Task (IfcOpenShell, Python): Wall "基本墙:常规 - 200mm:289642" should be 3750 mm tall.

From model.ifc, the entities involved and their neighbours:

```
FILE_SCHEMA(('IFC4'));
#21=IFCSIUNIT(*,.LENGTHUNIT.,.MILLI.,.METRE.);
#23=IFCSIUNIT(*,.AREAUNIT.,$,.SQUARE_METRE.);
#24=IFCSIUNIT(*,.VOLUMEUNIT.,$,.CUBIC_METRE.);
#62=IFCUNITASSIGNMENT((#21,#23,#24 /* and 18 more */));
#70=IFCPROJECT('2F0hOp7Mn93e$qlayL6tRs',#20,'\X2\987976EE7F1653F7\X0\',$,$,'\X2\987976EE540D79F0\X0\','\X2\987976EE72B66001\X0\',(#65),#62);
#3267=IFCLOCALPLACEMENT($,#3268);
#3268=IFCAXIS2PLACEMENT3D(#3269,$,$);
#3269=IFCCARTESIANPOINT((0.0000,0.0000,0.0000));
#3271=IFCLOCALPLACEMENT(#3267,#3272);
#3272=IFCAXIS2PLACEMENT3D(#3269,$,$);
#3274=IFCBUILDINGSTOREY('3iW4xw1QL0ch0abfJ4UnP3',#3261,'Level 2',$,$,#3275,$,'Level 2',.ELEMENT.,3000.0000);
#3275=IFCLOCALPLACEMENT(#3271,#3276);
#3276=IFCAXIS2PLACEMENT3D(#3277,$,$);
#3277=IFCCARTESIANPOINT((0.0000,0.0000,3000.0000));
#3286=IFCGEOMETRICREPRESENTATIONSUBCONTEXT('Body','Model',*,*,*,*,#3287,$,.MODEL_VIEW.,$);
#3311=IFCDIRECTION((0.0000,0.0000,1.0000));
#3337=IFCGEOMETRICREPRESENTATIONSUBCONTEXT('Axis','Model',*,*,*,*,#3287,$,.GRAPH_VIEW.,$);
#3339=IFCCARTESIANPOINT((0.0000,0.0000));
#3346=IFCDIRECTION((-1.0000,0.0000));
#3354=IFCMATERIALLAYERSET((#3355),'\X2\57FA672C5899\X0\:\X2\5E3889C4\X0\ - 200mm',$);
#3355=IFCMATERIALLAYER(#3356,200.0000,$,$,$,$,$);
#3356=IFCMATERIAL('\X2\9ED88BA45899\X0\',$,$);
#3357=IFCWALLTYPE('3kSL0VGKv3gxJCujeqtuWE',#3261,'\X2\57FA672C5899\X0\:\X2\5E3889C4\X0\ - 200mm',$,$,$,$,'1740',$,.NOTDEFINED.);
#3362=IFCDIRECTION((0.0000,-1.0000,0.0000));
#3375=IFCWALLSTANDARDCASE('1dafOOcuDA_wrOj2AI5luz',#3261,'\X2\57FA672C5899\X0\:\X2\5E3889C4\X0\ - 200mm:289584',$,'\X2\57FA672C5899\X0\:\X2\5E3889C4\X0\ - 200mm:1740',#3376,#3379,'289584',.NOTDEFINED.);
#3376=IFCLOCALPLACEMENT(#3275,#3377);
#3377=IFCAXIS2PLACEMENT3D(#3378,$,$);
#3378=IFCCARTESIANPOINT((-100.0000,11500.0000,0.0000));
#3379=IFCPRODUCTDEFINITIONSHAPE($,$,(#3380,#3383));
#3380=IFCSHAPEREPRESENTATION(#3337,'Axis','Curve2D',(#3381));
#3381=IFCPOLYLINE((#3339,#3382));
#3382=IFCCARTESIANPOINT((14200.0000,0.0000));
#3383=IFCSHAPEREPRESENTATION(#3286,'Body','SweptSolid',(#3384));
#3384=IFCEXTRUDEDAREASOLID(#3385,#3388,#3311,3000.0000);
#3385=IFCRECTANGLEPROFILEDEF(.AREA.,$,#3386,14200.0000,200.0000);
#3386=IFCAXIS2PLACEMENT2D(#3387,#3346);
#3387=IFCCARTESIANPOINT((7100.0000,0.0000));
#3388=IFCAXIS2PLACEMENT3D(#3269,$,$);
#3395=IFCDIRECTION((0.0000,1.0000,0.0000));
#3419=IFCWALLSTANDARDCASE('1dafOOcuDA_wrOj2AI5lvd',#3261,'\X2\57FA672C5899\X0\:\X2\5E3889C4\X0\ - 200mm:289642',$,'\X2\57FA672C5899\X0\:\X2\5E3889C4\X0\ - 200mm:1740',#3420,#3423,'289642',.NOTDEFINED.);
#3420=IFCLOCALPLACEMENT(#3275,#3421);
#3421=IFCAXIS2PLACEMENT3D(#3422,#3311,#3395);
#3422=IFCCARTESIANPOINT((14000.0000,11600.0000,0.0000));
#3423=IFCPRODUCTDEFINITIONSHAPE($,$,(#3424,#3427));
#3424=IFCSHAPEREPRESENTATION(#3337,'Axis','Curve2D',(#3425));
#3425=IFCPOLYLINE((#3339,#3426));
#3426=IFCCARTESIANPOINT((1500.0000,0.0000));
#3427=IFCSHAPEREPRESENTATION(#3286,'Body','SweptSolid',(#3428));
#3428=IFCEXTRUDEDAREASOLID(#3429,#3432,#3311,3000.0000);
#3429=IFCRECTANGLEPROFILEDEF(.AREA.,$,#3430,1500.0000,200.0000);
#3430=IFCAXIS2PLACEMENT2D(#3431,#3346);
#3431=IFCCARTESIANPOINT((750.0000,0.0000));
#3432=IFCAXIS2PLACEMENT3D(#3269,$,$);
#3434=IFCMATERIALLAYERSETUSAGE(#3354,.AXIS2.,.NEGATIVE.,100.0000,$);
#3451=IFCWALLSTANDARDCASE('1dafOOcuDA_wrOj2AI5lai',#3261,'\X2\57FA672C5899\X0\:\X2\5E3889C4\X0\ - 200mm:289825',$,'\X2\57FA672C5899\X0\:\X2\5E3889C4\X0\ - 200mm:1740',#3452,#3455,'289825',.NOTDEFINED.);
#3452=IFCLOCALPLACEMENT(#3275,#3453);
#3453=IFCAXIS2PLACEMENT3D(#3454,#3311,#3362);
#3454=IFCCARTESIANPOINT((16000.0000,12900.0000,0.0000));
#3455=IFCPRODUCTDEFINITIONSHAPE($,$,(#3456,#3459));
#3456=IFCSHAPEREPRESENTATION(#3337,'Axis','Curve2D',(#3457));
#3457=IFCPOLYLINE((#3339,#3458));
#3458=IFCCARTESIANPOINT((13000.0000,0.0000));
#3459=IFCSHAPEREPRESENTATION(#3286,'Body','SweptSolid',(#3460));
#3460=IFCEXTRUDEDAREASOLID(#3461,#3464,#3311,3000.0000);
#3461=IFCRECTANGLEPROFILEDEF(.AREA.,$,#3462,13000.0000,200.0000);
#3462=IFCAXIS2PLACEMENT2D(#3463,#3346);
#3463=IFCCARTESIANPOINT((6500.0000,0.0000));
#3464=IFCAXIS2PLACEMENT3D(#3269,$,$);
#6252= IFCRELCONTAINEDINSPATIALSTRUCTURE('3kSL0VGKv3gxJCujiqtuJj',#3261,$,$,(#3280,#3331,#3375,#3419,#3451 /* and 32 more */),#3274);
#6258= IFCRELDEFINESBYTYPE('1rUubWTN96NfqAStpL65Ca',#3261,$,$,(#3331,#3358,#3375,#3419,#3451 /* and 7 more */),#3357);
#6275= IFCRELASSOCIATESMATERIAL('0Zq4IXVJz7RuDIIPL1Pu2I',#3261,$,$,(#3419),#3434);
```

```python
import ifcopenshell
import ifcopenshell.geom
import ifcopenshell.util.representation
import ifcopenshell.util.shape

model = ifcopenshell.open("model.ifc")
settings = ifcopenshell.geom.settings()


def volume(element):
    """Net volume in cubic metres, openings subtracted."""
    shape = ifcopenshell.geom.create_shape(settings, element)
    return ifcopenshell.util.shape.get_volume(shape.geometry)


wall = model.by_guid("1dafOOcuDA_wrOj2AI5lvd")
before = volume(wall)

body = ifcopenshell.util.representation.get_representation(wall, "Model", "Body")
solid = body.Items[0]
old_height = solid.Depth
solid.Depth = 3750.0
after = volume(wall)

print(f"height {old_height:g} -> {solid.Depth:g}, volume {before:.3f} -> {after:.3f} m3")

model.write("model-out.ifc")
```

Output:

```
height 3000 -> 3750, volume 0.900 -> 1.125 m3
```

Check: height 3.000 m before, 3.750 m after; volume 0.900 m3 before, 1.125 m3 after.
